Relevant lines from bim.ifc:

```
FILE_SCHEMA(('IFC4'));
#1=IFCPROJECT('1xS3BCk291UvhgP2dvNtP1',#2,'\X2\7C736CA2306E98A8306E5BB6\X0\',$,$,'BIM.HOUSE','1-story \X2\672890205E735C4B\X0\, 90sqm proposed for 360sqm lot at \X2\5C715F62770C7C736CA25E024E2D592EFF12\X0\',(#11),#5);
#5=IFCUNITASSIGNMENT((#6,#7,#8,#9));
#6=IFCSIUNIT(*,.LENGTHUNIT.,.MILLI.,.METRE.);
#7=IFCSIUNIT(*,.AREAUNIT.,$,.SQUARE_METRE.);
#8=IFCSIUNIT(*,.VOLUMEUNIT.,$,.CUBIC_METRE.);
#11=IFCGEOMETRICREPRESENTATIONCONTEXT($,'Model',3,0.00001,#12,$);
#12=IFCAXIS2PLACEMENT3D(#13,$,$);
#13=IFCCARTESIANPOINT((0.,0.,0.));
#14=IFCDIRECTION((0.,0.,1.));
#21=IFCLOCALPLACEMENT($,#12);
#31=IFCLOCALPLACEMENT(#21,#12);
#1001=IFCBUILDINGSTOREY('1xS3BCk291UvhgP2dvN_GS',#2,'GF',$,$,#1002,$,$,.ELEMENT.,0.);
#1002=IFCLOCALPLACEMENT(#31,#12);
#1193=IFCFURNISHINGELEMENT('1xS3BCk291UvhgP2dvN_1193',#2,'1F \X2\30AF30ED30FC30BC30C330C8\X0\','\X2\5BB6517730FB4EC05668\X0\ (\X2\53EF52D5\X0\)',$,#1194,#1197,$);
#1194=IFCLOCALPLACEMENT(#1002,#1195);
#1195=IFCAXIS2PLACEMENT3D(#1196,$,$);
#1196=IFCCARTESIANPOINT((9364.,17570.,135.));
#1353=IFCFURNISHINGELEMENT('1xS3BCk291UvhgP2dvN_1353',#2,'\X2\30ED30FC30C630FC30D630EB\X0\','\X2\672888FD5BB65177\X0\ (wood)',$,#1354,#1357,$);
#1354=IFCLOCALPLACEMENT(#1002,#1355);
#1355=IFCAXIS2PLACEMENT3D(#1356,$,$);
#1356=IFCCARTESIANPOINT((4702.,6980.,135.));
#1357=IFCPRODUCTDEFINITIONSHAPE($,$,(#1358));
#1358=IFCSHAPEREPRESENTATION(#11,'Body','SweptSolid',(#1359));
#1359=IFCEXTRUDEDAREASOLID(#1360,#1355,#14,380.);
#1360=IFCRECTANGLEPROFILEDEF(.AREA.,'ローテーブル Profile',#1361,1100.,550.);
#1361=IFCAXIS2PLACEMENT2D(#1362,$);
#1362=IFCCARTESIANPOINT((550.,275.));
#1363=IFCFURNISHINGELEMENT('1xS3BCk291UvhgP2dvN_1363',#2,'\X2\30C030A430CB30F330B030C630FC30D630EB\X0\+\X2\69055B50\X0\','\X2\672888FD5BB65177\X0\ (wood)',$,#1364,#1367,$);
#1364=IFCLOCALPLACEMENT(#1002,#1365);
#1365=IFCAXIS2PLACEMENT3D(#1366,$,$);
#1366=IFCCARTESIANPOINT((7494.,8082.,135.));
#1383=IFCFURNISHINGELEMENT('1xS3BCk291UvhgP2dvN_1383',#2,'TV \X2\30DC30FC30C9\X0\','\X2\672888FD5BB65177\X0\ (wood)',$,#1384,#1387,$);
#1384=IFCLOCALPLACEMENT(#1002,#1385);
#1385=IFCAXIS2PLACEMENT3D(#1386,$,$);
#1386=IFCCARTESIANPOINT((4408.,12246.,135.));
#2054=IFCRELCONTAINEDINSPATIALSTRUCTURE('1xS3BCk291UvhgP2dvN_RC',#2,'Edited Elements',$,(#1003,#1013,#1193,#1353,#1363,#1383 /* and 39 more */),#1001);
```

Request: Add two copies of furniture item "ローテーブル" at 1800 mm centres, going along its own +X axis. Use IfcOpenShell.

```python
import ifcopenshell
import ifcopenshell.api.geometry
import ifcopenshell.api.root
import ifcopenshell.util.element
import ifcopenshell.util.placement

model = ifcopenshell.open("bim.ifc")


def reuse_history(source, copy):
    """copy_class also copies each property set's owner history, people and application; keep the originals."""
    for rel in copy.IsDefinedBy:
        if rel.is_a("IfcRelDefinesByProperties") and (history := rel.RelatingPropertyDefinition.OwnerHistory):
            rel.RelatingPropertyDefinition.OwnerHistory = source.OwnerHistory
            ifcopenshell.util.element.remove_deep2(model, history)


source = model.by_guid("1xS3BCk291UvhgP2dvN_1353")
base = ifcopenshell.util.placement.get_local_placement(source.ObjectPlacement)
step = base[:3, 0] * 1800.0

for i in range(1, 3):
    copy = ifcopenshell.api.root.copy_class(model, product=source)
    copy.Representation = ifcopenshell.util.element.copy_deep(
        model, source.Representation, exclude=["IfcGeometricRepresentationContext", "IfcRepresentationMap"]
    )
    reuse_history(source, copy)
    matrix = base.copy()
    matrix[:3, 3] += i * step
    print("added at", matrix[:3, 3].round(3) + 0.0)
    ifcopenshell.api.geometry.edit_object_placement(model, product=copy, matrix=matrix, is_si=False)

model.write("bim_v2.ifc")
```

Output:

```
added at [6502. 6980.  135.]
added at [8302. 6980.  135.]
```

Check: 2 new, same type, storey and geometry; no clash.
